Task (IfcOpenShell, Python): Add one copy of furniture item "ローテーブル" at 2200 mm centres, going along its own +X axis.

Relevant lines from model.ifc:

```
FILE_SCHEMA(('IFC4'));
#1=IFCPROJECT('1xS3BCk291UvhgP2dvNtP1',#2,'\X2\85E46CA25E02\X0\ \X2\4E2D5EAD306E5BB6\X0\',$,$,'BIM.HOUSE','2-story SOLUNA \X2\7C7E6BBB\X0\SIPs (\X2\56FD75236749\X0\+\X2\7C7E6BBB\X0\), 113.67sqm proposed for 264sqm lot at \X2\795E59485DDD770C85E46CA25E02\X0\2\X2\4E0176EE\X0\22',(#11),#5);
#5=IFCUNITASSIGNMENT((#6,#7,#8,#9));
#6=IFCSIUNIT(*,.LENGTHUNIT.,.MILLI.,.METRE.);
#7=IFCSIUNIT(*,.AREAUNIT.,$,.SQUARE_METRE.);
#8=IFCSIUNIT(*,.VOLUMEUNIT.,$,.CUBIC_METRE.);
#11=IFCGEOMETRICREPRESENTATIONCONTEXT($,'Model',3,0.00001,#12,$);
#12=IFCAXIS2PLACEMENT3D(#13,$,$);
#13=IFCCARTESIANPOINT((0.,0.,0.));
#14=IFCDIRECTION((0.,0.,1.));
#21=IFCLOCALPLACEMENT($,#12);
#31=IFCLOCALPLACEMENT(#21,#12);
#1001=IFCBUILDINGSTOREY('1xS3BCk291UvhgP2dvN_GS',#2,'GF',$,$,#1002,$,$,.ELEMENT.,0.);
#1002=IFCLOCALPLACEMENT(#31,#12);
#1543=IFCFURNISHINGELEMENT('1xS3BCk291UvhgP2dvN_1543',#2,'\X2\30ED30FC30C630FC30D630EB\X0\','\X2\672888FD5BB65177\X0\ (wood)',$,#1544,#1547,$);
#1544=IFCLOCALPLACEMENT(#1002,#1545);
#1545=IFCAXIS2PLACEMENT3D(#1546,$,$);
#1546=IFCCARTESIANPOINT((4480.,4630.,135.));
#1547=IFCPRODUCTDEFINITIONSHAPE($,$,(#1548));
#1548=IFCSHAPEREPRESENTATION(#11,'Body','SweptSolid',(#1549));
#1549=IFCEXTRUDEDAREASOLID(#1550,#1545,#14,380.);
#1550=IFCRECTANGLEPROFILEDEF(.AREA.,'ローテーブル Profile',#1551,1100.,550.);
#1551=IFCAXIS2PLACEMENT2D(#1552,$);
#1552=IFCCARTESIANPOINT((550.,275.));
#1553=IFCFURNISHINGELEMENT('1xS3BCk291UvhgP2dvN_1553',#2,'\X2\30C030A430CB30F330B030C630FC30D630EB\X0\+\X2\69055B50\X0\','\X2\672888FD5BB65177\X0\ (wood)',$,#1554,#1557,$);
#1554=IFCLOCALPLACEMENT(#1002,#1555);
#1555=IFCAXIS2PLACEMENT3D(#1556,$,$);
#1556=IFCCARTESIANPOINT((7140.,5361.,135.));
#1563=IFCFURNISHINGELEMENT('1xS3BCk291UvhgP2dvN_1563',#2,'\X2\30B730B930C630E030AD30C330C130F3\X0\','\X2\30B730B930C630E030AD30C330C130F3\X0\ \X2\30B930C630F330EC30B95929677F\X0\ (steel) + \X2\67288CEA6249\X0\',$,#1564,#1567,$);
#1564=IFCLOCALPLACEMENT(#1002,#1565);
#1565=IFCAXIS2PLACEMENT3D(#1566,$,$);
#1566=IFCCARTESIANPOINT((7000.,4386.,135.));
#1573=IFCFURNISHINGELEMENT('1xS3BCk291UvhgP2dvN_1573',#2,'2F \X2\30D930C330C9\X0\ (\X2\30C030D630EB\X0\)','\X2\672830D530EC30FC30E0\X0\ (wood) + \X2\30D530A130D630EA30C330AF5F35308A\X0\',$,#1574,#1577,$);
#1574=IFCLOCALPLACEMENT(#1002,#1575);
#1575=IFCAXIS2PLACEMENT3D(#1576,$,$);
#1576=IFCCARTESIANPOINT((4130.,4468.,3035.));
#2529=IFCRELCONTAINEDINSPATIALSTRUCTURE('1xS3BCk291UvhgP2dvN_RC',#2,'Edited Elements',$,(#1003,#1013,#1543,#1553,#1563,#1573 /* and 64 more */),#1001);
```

```python
import ifcopenshell
import ifcopenshell.api.geometry
import ifcopenshell.api.root
import ifcopenshell.util.element
import ifcopenshell.util.placement
import ifcopenshell.util.unit

model = ifcopenshell.open("model.ifc")
unit_scale = ifcopenshell.util.unit.calculate_unit_scale(model)


def reuse_history(source, copy):
    """copy_class also copies each property set's owner history, people and application; keep the originals."""
    for rel in copy.IsDefinedBy:
        if rel.is_a("IfcRelDefinesByProperties") and (history := rel.RelatingPropertyDefinition.OwnerHistory):
            rel.RelatingPropertyDefinition.OwnerHistory = source.OwnerHistory
            ifcopenshell.util.element.remove_deep2(model, history)


source = model.by_guid("1xS3BCk291UvhgP2dvN_1543")
base = ifcopenshell.util.placement.get_local_placement(source.ObjectPlacement)
step = base[:3, 0] * 2.2 / unit_scale

for i in range(1, 2):
    copy = ifcopenshell.api.root.copy_class(model, product=source)
    copy.Representation = ifcopenshell.util.element.copy_deep(
        model, source.Representation, exclude=["IfcGeometricRepresentationContext", "IfcRepresentationMap"]
    )
    reuse_history(source, copy)
    matrix = base.copy()
    matrix[:3, 3] += i * step
    print("added at", matrix[:3, 3].round(3) + 0.0)
    ifcopenshell.api.geometry.edit_object_placement(model, product=copy, matrix=matrix, is_si=False)

model.write("model_v2.ifc")
```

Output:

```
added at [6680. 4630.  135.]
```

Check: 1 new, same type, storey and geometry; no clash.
